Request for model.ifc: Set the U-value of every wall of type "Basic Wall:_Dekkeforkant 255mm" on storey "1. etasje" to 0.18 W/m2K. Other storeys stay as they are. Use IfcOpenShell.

First a look at what the model holds.

```python
import ifcopenshell
import ifcopenshell.util.element

model = ifcopenshell.open("model.ifc")
print(model.schema)
storey = next(s for s in model.by_type("IfcBuildingStorey") if s.Name == "1. etasje")
walls = [e for e in ifcopenshell.util.element.get_decomposition(storey) if e.is_a("IfcWall")]
seen = {}
for e in walls:
    element_type = ifcopenshell.util.element.get_type(e)
    key = (element_type.Name if element_type != e and element_type else None, ifcopenshell.util.element.get_pset(e, "Pset_WallCommon", "ThermalTransmittance"))
    seen[key] = seen.get(key, 0) + 1
for (name, value), count in sorted(seen.items(), key=str):
    print(count, "x", name, "|", value)
```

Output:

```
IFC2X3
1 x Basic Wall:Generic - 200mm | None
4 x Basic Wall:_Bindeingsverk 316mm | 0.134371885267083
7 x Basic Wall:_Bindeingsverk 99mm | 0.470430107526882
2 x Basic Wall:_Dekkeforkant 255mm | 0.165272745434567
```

```python
import ifcopenshell
import ifcopenshell.api.pset
import ifcopenshell.util.element

model = ifcopenshell.open("model.ifc")

storey = next(s for s in model.by_type("IfcBuildingStorey") if s.Name == "1. etasje")
walls = [e for e in ifcopenshell.util.element.get_decomposition(storey) if e.is_a("IfcWall")]

count = 0
for e in walls:
    element_type = ifcopenshell.util.element.get_type(e)
    if element_type in (None, e) or element_type.Name != "Basic Wall:_Dekkeforkant 255mm":
        continue
    # add_pset returns the element's existing set when there is one.
    pset = ifcopenshell.api.pset.add_pset(model, product=e, name="Pset_WallCommon")
    ifcopenshell.api.pset.edit_pset(model, pset=pset, properties={"ThermalTransmittance": 0.18})
    count += 1

print(count, "walls updated")

model.write("model_v2.ifc")
```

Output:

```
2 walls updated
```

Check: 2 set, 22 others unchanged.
